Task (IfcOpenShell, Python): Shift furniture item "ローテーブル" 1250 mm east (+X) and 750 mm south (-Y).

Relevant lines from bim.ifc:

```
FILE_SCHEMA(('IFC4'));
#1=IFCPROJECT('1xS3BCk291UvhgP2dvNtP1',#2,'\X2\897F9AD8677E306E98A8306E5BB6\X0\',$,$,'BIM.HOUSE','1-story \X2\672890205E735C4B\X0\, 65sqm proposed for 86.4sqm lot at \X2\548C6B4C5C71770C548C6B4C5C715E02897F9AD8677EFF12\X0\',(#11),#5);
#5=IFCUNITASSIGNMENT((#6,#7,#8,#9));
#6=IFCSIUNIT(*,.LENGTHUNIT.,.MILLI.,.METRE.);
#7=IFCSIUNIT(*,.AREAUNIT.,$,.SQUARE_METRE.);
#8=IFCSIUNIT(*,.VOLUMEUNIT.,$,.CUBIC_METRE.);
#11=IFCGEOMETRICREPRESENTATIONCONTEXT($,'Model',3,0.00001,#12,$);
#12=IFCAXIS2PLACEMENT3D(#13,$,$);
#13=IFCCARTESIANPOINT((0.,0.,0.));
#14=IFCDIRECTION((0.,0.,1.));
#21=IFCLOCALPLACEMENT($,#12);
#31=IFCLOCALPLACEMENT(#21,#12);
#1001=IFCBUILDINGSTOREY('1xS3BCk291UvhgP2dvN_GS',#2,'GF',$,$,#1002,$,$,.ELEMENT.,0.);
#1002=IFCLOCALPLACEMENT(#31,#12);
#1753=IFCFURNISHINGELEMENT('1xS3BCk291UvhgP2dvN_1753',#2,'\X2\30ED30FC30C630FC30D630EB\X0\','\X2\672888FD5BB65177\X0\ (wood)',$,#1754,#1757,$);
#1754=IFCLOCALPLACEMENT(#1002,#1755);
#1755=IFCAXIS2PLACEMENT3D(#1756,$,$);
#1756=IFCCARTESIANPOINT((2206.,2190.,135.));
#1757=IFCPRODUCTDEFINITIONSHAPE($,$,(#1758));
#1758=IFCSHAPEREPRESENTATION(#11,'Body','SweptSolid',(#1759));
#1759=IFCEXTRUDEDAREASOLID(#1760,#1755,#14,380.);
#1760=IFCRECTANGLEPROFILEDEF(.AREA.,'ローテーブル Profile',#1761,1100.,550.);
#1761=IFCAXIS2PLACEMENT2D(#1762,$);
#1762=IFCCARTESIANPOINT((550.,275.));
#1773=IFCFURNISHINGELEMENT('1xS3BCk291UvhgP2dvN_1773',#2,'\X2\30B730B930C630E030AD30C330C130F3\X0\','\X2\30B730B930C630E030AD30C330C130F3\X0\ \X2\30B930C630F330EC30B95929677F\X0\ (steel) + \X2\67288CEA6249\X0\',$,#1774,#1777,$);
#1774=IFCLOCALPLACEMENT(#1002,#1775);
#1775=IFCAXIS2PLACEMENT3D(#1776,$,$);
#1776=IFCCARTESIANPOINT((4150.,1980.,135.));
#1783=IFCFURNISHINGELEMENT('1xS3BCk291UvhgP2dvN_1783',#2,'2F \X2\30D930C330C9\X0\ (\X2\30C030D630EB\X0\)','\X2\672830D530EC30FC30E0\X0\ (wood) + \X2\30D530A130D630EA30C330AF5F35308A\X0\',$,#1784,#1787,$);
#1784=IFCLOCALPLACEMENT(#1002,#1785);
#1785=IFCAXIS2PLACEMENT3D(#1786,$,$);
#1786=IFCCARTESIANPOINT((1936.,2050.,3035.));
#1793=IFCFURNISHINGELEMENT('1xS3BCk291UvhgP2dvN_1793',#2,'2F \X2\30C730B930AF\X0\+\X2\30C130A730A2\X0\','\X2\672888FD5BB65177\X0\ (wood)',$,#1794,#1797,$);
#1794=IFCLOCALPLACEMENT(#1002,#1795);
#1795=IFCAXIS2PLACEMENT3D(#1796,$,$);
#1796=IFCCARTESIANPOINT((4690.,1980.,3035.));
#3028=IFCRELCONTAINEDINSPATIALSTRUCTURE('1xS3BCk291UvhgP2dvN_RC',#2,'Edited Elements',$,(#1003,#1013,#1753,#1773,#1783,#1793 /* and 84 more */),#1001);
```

```python
import ifcopenshell
import ifcopenshell.api.geometry
import ifcopenshell.util.placement
import ifcopenshell.util.unit

model = ifcopenshell.open("bim.ifc")
unit_scale = ifcopenshell.util.unit.calculate_unit_scale(model)

item = model.by_guid("1xS3BCk291UvhgP2dvN_1753")
matrix = ifcopenshell.util.placement.get_local_placement(item.ObjectPlacement)
matrix[0, 3] += 1.25 / unit_scale
matrix[1, 3] -= 0.75 / unit_scale
ifcopenshell.api.geometry.edit_object_placement(model, product=item, matrix=matrix, is_si=False)

print(ifcopenshell.util.placement.get_local_placement(item.ObjectPlacement).round(3) + 0.0)

model.write("bim_rev.ifc")
```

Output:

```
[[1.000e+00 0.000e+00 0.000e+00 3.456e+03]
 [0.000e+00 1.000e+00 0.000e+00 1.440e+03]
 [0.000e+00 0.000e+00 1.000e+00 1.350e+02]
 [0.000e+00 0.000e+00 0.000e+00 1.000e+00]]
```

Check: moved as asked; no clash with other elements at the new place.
